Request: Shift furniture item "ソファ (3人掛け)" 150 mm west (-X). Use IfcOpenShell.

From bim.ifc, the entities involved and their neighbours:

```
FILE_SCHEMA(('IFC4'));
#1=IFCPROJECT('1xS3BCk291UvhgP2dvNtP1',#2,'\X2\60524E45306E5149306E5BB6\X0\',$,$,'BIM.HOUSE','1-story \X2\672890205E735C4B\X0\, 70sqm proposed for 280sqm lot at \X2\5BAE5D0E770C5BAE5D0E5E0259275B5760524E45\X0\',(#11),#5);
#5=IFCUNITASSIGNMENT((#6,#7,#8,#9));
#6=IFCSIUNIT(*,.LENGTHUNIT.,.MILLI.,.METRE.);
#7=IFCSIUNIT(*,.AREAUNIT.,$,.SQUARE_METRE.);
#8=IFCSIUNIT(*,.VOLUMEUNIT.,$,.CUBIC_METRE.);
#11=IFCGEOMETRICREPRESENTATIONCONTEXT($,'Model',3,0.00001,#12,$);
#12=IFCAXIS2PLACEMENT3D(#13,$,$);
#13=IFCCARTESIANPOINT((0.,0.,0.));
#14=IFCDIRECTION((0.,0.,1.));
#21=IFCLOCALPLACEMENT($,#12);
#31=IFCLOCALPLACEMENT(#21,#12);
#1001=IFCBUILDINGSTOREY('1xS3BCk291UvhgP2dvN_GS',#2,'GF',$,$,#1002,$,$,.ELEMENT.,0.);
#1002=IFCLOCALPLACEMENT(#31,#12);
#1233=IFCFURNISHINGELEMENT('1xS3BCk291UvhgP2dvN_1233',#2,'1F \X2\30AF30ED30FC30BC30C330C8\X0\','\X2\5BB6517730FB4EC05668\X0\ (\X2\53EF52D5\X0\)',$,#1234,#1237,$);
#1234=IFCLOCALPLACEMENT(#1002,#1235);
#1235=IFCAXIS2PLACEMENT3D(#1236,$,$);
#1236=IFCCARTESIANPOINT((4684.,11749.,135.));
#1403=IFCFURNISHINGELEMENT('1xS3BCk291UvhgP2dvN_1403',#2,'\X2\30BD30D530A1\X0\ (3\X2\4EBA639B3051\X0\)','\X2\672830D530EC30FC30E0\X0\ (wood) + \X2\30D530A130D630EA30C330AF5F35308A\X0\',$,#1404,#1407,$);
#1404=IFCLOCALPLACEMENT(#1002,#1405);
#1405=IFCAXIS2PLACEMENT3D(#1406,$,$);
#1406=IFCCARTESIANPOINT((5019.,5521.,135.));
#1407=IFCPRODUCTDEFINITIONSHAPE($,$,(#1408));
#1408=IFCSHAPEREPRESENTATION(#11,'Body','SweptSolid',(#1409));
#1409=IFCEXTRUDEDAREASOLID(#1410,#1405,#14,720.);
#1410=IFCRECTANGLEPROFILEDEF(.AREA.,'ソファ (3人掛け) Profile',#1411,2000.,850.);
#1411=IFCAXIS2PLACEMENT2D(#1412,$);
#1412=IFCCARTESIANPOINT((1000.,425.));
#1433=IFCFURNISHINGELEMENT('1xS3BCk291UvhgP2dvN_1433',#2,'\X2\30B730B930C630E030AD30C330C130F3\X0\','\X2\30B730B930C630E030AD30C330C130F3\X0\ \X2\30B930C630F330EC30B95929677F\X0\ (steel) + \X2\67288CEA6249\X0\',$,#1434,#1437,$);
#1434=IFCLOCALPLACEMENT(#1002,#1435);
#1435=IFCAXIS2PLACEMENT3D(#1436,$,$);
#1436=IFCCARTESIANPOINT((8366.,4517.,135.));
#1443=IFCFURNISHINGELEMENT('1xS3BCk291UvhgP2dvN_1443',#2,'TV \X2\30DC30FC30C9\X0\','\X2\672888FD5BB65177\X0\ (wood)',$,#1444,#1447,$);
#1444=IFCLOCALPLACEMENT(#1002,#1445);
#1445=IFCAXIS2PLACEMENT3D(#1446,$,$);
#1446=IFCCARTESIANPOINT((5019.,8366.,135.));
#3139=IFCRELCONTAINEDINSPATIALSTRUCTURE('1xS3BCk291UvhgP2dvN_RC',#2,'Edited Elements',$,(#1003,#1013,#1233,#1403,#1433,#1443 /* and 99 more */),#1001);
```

```python
import ifcopenshell
import ifcopenshell.api.geometry
import ifcopenshell.util.placement

model = ifcopenshell.open("bim.ifc")

item = model.by_guid("1xS3BCk291UvhgP2dvN_1403")
matrix = ifcopenshell.util.placement.get_local_placement(item.ObjectPlacement)
matrix[0, 3] -= 150.0
ifcopenshell.api.geometry.edit_object_placement(model, product=item, matrix=matrix, is_si=False)

print(ifcopenshell.util.placement.get_local_placement(item.ObjectPlacement).round(3) + 0.0)

model.write("bim_updated.ifc")
```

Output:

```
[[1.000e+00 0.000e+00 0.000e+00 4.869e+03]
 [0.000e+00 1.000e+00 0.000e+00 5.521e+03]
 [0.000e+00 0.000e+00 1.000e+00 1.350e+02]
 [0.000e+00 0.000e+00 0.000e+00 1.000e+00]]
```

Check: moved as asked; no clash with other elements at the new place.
